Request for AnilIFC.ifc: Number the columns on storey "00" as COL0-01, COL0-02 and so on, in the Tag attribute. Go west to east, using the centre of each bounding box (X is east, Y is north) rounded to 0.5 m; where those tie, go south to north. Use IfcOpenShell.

First a look at what the model holds.

```python
import ifcopenshell
import ifcopenshell.util.element
import ifcopenshell.util.placement

model = ifcopenshell.open("AnilIFC.ifc")
print(model.schema)
storey = next(s for s in model.by_type("IfcBuildingStorey") if s.Name == "00")
columns = [e for e in ifcopenshell.util.element.get_decomposition(storey) if e.is_a("IfcColumn")]
for e in sorted(columns, key=lambda e: e.id()):
    origin = ifcopenshell.util.placement.get_local_placement(e.ObjectPlacement)[:3, 3]
    print(e.id(), e.Tag, e.Name, origin.round(2) + 0.0, sep=" | ")
```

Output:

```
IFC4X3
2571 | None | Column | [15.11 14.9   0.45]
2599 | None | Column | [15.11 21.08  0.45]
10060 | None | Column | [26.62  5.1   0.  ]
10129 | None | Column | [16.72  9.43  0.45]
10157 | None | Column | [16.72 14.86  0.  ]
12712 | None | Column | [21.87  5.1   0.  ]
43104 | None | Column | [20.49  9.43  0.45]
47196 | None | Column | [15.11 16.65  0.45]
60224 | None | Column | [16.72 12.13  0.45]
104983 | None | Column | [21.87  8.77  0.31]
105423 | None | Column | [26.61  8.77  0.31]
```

```python
import ifcopenshell
import ifcopenshell.geom
import ifcopenshell.util.element
import ifcopenshell.util.shape

model = ifcopenshell.open("AnilIFC.ifc")
settings = ifcopenshell.geom.settings()
settings.set("use-world-coords", True)


def centre(element):
    shape = ifcopenshell.geom.create_shape(settings, element)
    return ifcopenshell.util.shape.get_bbox_centroid(shape.geometry)


storey = next(s for s in model.by_type("IfcBuildingStorey") if s.Name == "00")
columns = [e for e in ifcopenshell.util.element.get_decomposition(storey) if e.is_a("IfcColumn")]

# Insertion points can sit at a corner or the storey origin, so sort by the geometry (in metres).
centres = {e: centre(e) for e in columns}
columns.sort(key=lambda e: (round(centres[e][0] / 0.5), centres[e][1]))

for i, e in enumerate(columns, start=1):
    number = f"COL0-{i:02d}"
    e.Tag = number
    print(e.id(), number)

model.write("AnilIFC_updated.ifc")
```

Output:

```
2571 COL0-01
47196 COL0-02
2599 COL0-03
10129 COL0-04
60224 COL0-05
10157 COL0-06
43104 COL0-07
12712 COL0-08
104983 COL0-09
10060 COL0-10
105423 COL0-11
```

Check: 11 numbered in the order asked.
